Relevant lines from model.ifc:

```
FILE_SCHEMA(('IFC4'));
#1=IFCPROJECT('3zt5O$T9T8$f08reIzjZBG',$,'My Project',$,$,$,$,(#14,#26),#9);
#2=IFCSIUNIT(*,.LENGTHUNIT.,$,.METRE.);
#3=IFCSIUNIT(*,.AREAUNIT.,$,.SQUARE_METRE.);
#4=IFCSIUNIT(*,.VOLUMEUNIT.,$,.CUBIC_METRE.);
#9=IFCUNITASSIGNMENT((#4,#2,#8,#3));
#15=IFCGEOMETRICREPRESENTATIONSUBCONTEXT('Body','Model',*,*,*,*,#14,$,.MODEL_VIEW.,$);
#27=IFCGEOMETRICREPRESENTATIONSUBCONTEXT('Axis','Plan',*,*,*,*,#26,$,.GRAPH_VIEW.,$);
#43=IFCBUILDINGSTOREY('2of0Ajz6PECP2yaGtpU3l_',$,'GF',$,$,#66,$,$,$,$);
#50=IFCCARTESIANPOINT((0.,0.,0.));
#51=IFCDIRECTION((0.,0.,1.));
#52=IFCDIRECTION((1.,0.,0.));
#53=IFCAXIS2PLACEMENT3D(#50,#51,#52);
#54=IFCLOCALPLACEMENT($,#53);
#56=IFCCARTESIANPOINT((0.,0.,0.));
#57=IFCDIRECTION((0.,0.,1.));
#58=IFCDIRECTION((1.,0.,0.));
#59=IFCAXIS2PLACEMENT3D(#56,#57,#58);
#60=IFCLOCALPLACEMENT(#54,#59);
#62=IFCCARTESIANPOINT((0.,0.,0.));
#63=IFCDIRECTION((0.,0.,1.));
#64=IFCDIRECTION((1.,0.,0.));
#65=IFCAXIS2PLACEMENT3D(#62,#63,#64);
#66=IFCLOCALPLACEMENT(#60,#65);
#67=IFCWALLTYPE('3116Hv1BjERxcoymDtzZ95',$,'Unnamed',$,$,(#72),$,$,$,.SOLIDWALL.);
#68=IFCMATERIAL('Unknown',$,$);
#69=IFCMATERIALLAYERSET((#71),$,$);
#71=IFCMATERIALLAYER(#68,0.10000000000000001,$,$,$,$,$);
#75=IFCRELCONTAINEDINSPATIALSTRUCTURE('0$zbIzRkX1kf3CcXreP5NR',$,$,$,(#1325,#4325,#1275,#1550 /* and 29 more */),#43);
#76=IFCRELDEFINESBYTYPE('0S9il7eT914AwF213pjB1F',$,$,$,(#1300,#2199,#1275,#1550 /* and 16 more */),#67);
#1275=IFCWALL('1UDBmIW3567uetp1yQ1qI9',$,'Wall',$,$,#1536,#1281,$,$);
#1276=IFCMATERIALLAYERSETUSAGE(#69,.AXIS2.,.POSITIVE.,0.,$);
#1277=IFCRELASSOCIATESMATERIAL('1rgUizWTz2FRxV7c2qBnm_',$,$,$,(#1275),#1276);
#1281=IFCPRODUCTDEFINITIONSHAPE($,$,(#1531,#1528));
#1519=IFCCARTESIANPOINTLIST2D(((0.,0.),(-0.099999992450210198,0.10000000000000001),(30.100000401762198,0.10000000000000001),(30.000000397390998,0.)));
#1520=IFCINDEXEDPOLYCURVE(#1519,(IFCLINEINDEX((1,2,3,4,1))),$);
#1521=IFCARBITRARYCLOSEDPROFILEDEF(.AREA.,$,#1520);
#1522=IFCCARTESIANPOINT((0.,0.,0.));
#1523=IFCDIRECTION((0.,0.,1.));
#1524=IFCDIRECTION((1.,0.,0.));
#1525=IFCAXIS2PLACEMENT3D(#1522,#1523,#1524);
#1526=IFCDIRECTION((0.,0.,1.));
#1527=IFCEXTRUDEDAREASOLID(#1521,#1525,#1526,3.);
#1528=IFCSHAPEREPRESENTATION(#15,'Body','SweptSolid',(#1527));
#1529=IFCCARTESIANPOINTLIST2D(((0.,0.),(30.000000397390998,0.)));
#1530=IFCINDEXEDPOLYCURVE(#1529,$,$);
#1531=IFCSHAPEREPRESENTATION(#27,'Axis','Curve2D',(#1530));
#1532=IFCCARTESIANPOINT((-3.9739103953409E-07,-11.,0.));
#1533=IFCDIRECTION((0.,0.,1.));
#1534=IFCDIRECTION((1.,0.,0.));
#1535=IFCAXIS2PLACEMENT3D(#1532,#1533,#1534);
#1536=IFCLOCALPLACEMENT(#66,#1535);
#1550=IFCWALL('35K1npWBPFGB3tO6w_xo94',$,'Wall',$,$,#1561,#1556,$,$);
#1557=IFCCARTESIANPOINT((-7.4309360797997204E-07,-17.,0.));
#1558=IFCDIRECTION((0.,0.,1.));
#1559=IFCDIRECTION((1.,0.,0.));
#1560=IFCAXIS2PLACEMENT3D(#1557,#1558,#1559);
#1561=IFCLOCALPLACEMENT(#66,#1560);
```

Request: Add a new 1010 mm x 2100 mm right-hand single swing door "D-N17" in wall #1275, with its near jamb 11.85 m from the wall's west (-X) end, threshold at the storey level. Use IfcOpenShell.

```python
import numpy as np
import ifcopenshell
import ifcopenshell.api.feature
import ifcopenshell.api.geometry
import ifcopenshell.api.root
import ifcopenshell.api.spatial
import ifcopenshell.geom
import ifcopenshell.util.element
import ifcopenshell.util.placement
import ifcopenshell.util.representation
import ifcopenshell.util.shape
import ifcopenshell.util.unit

model = ifcopenshell.open("model.ifc")
unit_scale = ifcopenshell.util.unit.calculate_unit_scale(model)
settings = ifcopenshell.geom.settings()


def volume(element):
    """Net volume in cubic metres, openings subtracted."""
    shape = ifcopenshell.geom.create_shape(settings, element)
    return ifcopenshell.util.shape.get_volume(shape.geometry)


wall = model.by_guid("1UDBmIW3567uetp1yQ1qI9")
storey = ifcopenshell.util.element.get_container(wall, ifc_class="IfcBuildingStorey")
context = ifcopenshell.util.representation.get_context(model, "Model", "Body", "MODEL_VIEW")
before = volume(wall)

width, height, from_end, sill = 1.01, 2.1, 11.85, 0.0  # metres

# The wall runs along its own X axis, and the end named is its -X end.
wall_shape = ifcopenshell.geom.create_shape(settings, wall)
x, y, z = ifcopenshell.util.shape.get_vertices(wall_shape.geometry).T
start = x.min() + from_end
face, thickness = float(y.min()), float(y.max() - y.min())
wall_matrix = ifcopenshell.util.placement.get_local_placement(wall.ObjectPlacement)
level = ifcopenshell.util.placement.get_local_placement(storey.ObjectPlacement)[2, 3]


def in_wall(x, y):
    """Placement at x, y metres in the wall's axes, at sill height."""
    matrix = wall_matrix.copy()
    matrix[:, 3] = wall_matrix @ np.array([x / unit_scale, y / unit_scale, 0.0, 1.0])
    matrix[2, 3] = level + sill / unit_scale
    return matrix


# Opening: a box that overshoots both wall faces by 50 mm.
opening = ifcopenshell.api.root.create_entity(model, ifc_class="IfcOpeningElement", predefined_type="OPENING")
box = ifcopenshell.api.geometry.add_wall_representation(
    model, context=context, length=width, height=height, thickness=thickness + 0.1
)
ifcopenshell.api.geometry.assign_representation(model, product=opening, representation=box)
ifcopenshell.api.geometry.edit_object_placement(model, product=opening, matrix=in_wall(start, face - 0.05), is_si=False)
ifcopenshell.api.feature.add_feature(model, feature=opening, element=wall)

door = ifcopenshell.api.root.create_entity(model, ifc_class="IfcDoor", name="D-N17", predefined_type="DOOR")
door.OverallWidth, door.OverallHeight = width / unit_scale, height / unit_scale
door.OperationType = "SINGLE_SWING_RIGHT"
body = ifcopenshell.api.geometry.add_door_representation(
    model,
    context=context,
    overall_width=door.OverallWidth,
    overall_height=door.OverallHeight,
    operation_type="SINGLE_SWING_RIGHT",
    lining_properties={"LiningDepth": thickness / unit_scale, "ThresholdDepth": thickness / unit_scale},
)
ifcopenshell.api.geometry.assign_representation(model, product=door, representation=body)
ifcopenshell.api.spatial.assign_container(model, products=[door], relating_structure=storey)
ifcopenshell.api.feature.add_filling(model, opening=opening, element=door)

# The lining spans the wall, so the door starts at the wall face.
ifcopenshell.api.geometry.edit_object_placement(model, product=door, matrix=in_wall(start, face), is_si=False)

after = volume(wall)

print(f"wall volume {before:.3f} -> {after:.3f} m3")

model.write("model_edited.ifc")
```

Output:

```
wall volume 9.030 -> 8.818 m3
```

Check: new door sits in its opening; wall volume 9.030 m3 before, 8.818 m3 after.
